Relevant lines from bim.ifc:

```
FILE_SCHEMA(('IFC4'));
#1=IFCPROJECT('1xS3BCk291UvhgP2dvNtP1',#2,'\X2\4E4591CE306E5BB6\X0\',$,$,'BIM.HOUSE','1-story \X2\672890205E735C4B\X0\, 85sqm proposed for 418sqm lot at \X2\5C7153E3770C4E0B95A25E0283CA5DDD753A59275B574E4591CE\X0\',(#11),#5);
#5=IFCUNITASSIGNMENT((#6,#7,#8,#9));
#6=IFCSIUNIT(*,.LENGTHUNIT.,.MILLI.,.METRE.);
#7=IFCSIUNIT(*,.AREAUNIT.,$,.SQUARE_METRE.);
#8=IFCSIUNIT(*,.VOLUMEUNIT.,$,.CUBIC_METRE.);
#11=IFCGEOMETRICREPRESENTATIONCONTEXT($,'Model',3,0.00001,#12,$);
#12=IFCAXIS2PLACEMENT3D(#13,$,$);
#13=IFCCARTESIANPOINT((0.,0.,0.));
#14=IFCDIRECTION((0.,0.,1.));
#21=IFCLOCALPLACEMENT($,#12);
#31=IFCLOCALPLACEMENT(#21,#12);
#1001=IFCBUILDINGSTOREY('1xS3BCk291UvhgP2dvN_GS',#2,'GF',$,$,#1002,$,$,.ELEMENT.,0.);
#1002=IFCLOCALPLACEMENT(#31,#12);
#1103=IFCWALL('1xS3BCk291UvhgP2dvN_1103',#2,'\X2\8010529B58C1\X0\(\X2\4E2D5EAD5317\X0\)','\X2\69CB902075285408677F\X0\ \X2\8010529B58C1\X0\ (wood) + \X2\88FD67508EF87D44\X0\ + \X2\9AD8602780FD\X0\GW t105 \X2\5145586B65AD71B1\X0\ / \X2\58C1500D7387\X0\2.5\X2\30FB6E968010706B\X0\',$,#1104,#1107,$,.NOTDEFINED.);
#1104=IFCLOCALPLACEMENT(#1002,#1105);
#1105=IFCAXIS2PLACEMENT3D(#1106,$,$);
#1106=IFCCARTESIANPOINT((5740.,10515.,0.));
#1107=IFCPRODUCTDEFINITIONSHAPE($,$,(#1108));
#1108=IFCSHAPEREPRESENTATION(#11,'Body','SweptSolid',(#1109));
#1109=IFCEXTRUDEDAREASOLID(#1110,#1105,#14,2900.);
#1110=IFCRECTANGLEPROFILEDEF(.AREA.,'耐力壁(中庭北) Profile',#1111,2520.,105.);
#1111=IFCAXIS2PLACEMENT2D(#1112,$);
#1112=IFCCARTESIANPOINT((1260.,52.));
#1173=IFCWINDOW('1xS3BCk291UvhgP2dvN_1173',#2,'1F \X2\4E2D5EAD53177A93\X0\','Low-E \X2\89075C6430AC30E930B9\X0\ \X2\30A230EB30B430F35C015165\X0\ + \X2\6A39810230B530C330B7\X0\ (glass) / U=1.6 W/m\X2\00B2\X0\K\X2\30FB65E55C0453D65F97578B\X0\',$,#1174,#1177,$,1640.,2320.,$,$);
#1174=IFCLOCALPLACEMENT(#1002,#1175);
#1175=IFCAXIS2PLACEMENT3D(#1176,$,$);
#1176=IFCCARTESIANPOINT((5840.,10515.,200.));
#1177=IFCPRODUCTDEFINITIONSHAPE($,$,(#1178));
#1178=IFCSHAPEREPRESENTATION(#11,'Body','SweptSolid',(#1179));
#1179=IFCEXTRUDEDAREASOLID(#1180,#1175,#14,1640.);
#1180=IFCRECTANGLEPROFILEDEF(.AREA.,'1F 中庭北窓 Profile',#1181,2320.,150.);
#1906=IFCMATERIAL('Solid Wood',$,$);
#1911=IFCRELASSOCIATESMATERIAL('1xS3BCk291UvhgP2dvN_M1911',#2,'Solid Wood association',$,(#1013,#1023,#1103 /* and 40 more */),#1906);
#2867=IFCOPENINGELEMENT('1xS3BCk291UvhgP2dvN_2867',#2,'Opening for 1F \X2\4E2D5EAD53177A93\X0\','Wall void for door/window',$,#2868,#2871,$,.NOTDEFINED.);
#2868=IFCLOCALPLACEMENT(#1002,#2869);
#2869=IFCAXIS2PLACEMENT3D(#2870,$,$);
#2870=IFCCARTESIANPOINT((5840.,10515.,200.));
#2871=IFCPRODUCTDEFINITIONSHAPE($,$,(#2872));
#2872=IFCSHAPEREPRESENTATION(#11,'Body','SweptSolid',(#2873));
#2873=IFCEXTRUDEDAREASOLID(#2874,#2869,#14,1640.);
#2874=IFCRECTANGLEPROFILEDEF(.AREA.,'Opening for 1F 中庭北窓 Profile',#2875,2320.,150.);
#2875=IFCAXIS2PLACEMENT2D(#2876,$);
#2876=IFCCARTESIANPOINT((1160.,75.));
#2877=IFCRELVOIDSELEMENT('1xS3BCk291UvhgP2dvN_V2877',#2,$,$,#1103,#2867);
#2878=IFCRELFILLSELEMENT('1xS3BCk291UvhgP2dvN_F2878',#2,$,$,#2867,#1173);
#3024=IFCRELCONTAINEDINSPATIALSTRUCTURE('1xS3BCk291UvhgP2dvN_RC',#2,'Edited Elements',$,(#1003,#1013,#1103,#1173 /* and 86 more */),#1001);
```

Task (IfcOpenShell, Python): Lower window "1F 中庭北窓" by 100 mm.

```python
import numpy as np
import ifcopenshell
import ifcopenshell.api.geometry
import ifcopenshell.util.placement
import ifcopenshell.util.unit

model = ifcopenshell.open("bim.ifc")
unit_scale = ifcopenshell.util.unit.calculate_unit_scale(model)

window = model.by_id(1173)
opening = window.FillsVoids[0].RelatingOpeningElement
dz = -100.0

shift = np.array([0.0, 0.0, dz])
# The window is not placed relative to its opening, so move both.
for product in (opening, window):
    matrix = ifcopenshell.util.placement.get_local_placement(product.ObjectPlacement)
    matrix[:3, 3] += shift
    ifcopenshell.api.geometry.edit_object_placement(model, product=product, matrix=matrix, is_si=False)

print(f"moved by {dz * unit_scale:+.3f} m")

model.write("bim_edited.ifc")
```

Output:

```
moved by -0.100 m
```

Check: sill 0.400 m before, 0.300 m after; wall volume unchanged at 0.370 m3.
